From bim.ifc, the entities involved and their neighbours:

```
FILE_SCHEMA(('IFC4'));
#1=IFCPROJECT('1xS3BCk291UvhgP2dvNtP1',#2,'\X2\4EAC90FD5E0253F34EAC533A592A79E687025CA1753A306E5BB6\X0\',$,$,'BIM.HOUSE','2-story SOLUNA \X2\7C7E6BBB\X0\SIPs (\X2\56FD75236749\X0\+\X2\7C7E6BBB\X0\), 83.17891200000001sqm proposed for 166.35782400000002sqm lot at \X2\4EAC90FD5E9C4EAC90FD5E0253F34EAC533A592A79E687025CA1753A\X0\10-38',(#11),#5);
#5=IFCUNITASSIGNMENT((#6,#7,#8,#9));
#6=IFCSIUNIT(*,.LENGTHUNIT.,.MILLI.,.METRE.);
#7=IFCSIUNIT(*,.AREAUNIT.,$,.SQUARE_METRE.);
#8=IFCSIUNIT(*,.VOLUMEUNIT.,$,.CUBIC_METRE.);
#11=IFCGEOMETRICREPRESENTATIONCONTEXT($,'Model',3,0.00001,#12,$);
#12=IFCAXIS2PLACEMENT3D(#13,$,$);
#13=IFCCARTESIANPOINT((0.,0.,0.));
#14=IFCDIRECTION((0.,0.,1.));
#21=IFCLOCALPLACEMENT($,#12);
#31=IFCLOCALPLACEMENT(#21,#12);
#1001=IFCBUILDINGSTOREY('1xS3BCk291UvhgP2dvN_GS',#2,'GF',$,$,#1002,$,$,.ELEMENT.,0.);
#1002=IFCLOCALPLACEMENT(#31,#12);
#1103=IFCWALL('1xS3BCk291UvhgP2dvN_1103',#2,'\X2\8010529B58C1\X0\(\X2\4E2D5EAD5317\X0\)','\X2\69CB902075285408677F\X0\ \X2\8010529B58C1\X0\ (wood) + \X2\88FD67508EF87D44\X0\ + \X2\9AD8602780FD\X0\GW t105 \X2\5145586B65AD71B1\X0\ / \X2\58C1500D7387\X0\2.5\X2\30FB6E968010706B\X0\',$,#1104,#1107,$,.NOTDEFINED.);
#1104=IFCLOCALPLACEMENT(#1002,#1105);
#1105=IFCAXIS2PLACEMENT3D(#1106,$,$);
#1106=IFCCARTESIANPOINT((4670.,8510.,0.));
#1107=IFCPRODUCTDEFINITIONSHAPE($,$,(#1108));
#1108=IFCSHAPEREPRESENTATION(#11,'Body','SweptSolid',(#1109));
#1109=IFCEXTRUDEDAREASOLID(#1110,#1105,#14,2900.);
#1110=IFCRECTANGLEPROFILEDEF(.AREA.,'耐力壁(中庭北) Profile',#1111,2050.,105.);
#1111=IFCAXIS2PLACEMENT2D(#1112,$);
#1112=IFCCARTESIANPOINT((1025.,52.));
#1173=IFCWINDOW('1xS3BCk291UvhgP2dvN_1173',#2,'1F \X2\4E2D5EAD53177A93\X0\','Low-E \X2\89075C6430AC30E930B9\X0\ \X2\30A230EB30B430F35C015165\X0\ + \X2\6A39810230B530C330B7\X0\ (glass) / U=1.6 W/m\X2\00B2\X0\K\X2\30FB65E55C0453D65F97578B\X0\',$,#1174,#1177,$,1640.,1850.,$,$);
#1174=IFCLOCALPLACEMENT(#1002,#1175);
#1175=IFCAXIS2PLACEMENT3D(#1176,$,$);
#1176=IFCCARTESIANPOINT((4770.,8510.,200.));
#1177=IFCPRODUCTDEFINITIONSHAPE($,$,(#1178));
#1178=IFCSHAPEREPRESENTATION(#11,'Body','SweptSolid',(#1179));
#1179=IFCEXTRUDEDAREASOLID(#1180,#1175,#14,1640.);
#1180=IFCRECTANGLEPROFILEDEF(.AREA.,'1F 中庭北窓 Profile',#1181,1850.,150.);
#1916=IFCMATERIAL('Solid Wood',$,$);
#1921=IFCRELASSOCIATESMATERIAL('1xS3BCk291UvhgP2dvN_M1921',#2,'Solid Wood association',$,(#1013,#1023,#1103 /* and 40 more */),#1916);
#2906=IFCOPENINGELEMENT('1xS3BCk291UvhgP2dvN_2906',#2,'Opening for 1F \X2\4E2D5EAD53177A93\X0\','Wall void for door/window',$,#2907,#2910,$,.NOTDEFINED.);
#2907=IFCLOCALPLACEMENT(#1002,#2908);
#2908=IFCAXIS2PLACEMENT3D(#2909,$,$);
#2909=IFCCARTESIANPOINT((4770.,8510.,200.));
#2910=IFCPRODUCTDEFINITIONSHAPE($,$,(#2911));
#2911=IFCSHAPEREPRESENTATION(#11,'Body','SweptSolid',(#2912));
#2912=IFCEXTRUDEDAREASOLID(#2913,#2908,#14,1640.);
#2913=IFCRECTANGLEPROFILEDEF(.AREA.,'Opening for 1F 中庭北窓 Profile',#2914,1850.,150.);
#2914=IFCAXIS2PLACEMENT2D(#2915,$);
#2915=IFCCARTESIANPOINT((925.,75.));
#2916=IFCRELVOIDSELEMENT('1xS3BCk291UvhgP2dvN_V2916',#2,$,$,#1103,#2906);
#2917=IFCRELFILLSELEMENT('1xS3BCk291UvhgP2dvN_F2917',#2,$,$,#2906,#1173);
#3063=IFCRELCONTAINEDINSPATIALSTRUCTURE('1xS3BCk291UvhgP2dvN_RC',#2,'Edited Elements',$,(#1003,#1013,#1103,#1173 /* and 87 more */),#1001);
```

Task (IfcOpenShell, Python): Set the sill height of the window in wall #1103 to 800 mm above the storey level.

```python
import numpy as np
import ifcopenshell
import ifcopenshell.api.geometry
import ifcopenshell.geom
import ifcopenshell.util.element
import ifcopenshell.util.placement
import ifcopenshell.util.shape
import ifcopenshell.util.unit

model = ifcopenshell.open("bim.ifc")
unit_scale = ifcopenshell.util.unit.calculate_unit_scale(model)

window = model.by_guid("1xS3BCk291UvhgP2dvN_1173")
opening = window.FillsVoids[0].RelatingOpeningElement
storey = ifcopenshell.util.element.get_container(window, ifc_class="IfcBuildingStorey")
level = ifcopenshell.util.placement.get_local_placement(storey.ObjectPlacement)[2, 3]

# The opening's origin need not be at the sill, so measure its lowest point.
shape = ifcopenshell.geom.create_shape(ifcopenshell.geom.settings(), opening)
bottom = ifcopenshell.util.shape.get_shape_bottom_elevation(shape, shape.geometry) / unit_scale
dz = level + 0.8 / unit_scale - bottom

shift = np.array([0.0, 0.0, dz])
# The window is not placed relative to its opening, so move both.
for product in (opening, window):
    matrix = ifcopenshell.util.placement.get_local_placement(product.ObjectPlacement)
    matrix[:3, 3] += shift
    ifcopenshell.api.geometry.edit_object_placement(model, product=product, matrix=matrix, is_si=False)

print(f"moved by {dz * unit_scale:+.3f} m")

model.write("bim_v2.ifc")
```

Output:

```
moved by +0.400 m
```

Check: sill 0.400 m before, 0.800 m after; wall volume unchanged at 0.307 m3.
